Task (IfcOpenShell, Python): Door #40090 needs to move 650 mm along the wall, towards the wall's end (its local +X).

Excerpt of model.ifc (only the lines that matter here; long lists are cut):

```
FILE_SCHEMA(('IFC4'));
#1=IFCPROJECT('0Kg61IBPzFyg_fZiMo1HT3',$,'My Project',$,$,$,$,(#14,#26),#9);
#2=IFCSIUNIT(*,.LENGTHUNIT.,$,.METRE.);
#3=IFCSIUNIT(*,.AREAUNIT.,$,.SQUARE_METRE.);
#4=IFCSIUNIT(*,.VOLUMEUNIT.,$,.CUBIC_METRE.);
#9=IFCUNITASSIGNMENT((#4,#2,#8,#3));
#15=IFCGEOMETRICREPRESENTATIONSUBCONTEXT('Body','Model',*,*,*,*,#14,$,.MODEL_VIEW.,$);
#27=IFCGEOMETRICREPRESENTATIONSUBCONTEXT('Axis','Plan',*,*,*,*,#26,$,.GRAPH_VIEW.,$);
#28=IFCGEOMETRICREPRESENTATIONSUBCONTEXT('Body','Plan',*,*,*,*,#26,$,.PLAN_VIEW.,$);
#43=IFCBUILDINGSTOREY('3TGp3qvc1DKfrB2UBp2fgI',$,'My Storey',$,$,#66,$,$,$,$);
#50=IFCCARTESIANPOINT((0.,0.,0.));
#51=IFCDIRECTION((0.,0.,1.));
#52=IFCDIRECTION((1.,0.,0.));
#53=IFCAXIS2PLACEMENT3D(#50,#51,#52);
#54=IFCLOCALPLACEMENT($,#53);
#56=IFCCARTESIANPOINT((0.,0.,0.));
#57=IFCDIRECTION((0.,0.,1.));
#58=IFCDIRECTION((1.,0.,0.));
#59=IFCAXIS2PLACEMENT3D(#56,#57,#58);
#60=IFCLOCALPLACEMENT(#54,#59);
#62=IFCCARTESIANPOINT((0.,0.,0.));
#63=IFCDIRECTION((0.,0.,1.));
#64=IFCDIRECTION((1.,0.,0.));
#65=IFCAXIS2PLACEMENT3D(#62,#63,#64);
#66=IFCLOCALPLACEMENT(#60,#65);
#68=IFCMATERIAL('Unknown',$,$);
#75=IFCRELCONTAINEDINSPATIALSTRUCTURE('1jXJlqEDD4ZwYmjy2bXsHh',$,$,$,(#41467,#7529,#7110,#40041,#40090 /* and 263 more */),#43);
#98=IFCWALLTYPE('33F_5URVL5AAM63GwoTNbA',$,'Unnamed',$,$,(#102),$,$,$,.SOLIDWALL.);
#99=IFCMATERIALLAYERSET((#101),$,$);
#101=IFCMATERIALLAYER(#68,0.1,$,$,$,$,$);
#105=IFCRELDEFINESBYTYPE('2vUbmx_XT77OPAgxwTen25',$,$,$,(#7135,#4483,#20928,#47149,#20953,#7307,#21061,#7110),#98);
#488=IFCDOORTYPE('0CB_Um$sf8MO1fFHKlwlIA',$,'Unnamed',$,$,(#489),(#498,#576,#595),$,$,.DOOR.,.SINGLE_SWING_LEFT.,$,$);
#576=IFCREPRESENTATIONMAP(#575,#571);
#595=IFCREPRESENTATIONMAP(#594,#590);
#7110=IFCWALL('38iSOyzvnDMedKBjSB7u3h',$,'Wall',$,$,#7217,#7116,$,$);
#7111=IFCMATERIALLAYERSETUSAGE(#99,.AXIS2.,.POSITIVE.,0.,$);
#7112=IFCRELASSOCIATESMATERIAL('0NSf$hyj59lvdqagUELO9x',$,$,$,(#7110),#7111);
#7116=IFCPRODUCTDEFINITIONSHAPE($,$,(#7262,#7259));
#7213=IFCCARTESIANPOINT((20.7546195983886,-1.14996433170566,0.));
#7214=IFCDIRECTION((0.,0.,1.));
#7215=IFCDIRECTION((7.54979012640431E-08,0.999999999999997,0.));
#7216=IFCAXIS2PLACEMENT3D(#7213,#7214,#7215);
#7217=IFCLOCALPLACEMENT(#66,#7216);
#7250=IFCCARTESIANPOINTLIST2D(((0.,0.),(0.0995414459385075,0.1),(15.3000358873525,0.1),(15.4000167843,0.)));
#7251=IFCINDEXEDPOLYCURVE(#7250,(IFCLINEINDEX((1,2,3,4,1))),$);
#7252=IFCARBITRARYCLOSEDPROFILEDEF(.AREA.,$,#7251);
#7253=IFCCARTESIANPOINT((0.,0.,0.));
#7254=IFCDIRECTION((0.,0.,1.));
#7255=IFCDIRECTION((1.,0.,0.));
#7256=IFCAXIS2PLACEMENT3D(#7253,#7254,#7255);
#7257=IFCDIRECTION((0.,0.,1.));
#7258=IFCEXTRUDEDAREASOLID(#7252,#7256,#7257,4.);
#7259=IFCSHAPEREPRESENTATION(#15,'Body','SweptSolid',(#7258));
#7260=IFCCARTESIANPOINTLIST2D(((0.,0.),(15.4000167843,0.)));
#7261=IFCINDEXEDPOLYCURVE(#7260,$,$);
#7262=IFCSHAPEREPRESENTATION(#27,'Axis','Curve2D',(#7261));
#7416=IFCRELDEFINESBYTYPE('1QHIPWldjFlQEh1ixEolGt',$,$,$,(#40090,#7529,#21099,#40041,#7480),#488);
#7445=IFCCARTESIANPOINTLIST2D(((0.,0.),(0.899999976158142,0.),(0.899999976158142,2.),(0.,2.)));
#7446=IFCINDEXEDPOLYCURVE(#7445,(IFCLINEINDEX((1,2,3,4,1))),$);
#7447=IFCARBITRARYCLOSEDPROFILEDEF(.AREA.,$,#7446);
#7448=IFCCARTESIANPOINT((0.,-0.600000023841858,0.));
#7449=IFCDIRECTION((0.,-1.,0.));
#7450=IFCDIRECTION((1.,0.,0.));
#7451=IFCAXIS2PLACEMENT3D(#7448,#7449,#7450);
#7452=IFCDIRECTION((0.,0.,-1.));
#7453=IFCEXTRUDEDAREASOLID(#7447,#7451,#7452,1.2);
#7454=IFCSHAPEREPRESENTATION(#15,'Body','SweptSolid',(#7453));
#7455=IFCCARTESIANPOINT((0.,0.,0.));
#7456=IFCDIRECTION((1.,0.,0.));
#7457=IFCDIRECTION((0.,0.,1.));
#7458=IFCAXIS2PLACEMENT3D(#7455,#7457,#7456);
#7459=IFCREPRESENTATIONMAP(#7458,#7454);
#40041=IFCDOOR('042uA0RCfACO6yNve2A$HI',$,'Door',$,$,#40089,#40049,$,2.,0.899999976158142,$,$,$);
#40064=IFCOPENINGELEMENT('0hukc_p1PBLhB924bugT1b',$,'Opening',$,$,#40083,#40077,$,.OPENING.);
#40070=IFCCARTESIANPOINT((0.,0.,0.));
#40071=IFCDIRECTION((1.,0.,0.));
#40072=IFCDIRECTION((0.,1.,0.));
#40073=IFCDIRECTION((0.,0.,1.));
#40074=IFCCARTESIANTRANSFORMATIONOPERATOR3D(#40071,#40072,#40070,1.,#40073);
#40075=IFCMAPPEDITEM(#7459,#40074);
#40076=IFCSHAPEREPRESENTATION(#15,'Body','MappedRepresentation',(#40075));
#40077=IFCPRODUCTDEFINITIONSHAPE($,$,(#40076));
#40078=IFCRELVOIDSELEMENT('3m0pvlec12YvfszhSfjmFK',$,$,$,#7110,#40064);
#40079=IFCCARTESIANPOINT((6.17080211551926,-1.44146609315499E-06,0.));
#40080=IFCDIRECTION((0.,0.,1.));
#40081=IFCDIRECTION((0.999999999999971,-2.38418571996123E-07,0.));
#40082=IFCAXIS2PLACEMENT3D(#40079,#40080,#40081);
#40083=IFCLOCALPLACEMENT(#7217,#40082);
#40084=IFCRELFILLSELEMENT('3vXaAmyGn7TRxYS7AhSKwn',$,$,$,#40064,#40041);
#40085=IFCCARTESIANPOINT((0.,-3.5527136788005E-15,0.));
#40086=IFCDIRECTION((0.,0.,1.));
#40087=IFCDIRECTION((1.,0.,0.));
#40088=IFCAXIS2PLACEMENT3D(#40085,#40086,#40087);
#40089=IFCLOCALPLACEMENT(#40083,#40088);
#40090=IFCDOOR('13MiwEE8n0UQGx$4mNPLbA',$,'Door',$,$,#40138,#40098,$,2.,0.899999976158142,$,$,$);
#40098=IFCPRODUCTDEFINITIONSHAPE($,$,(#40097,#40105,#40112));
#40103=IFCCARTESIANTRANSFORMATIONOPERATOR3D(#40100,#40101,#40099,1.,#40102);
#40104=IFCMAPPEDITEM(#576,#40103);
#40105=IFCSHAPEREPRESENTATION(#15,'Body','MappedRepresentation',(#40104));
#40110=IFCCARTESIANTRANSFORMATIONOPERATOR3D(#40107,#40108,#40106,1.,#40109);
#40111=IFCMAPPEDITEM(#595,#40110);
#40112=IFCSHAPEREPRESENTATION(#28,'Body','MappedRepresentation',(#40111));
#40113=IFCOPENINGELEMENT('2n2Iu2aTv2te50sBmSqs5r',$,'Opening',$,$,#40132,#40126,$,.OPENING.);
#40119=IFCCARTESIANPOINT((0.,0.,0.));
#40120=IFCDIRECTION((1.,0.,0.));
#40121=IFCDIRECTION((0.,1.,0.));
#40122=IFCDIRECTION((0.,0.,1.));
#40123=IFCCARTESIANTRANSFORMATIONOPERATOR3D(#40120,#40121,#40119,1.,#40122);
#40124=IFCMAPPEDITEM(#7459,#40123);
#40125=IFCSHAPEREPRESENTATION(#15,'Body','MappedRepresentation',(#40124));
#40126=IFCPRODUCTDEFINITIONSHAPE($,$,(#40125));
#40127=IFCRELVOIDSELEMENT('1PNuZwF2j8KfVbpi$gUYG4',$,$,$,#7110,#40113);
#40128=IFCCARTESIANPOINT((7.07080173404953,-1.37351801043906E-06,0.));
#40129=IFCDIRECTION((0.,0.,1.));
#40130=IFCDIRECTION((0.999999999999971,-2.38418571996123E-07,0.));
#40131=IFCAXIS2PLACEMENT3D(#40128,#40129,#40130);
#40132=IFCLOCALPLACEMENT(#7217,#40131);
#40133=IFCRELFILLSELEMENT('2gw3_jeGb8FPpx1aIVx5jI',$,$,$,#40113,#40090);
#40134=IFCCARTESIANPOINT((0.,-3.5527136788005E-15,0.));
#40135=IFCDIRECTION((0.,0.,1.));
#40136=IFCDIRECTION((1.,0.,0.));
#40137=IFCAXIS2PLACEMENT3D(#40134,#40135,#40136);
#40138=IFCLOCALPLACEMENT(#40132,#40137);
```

```python
import ifcopenshell
import ifcopenshell.api.geometry
import ifcopenshell.util.placement
import ifcopenshell.util.unit

model = ifcopenshell.open("model.ifc")
unit_scale = ifcopenshell.util.unit.calculate_unit_scale(model)

door = model.by_id(40090)
opening = door.FillsVoids[0].RelatingOpeningElement
wall = opening.VoidsElements[0].RelatingBuildingElement

wall_matrix = ifcopenshell.util.placement.get_local_placement(wall.ObjectPlacement)
shift = wall_matrix[:3, 0] * 0.65 / unit_scale
before = ifcopenshell.util.placement.get_local_placement(door.ObjectPlacement)[:3, 3].copy()

# The door is placed relative to its opening, so it follows when the opening moves.
matrix = ifcopenshell.util.placement.get_local_placement(opening.ObjectPlacement)
matrix[:3, 3] += shift
ifcopenshell.api.geometry.edit_object_placement(
    model, product=opening, matrix=matrix, is_si=False, should_transform_children=True
)

after = ifcopenshell.util.placement.get_local_placement(door.ObjectPlacement)[:3, 3]
print("door moved by", (after - before).round(3) + 0.0)

model.write("model_edited.ifc")
```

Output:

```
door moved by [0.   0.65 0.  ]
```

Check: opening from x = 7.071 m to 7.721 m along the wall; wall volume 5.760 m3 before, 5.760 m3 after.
